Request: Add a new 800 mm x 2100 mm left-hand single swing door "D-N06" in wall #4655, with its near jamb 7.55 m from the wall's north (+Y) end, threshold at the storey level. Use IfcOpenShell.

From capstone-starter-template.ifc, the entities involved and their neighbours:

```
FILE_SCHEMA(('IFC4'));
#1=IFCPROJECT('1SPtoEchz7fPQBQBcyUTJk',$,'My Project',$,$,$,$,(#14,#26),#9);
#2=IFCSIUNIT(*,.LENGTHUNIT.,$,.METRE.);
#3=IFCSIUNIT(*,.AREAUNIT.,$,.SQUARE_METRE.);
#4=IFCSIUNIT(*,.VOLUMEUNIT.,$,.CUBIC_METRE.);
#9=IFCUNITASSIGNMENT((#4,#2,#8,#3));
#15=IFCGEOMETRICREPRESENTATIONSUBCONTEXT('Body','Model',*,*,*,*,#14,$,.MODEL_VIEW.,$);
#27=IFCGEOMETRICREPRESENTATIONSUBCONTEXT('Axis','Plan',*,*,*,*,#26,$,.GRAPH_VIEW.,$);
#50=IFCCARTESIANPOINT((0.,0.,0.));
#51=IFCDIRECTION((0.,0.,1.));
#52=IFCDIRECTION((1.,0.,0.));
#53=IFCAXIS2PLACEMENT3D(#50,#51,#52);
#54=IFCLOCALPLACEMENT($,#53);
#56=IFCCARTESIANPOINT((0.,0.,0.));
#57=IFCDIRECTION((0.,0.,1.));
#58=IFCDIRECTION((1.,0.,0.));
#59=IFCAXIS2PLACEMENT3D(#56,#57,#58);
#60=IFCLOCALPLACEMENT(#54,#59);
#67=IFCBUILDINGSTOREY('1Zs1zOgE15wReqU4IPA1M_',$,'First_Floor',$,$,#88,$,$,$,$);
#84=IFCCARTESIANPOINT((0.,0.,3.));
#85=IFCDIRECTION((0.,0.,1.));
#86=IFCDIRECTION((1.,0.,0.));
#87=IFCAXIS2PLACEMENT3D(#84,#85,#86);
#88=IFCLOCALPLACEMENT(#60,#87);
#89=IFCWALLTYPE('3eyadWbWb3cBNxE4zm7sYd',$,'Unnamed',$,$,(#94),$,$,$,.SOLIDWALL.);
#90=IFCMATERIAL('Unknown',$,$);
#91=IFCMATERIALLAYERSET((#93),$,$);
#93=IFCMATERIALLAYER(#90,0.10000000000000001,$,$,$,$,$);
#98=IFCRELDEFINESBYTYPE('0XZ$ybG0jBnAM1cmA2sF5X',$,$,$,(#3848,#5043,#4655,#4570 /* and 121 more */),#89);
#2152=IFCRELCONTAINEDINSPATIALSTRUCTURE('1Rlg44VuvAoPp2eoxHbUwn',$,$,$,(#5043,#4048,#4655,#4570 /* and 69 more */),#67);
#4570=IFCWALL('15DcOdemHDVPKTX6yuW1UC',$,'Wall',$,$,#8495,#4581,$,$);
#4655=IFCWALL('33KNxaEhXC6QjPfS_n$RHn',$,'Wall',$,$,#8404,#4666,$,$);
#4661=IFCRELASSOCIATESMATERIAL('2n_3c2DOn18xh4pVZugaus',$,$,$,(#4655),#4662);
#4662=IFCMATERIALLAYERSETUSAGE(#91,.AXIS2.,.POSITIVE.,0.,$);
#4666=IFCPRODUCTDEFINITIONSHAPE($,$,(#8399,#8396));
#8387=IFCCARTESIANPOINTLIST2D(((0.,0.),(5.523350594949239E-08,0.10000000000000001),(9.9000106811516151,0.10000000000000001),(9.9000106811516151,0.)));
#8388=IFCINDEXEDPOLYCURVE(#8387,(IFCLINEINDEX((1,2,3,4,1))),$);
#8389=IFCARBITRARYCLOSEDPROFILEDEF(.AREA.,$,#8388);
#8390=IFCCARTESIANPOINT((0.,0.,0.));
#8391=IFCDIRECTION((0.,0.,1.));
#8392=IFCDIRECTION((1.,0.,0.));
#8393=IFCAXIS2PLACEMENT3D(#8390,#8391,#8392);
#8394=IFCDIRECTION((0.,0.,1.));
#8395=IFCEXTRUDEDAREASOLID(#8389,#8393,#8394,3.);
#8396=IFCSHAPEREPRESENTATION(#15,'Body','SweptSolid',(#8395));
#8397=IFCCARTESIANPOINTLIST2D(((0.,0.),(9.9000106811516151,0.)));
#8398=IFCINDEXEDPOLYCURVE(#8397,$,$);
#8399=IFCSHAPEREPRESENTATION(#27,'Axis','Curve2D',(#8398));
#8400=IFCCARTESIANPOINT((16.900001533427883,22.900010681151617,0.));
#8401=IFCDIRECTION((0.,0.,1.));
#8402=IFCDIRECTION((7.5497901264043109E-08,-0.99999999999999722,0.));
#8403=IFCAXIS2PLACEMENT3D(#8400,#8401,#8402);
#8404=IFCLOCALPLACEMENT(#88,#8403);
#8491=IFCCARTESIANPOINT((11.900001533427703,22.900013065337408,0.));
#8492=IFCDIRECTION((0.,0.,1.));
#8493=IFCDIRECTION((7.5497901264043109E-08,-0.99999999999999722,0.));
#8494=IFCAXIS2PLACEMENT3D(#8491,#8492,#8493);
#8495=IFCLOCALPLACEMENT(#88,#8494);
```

```python
import numpy as np
import ifcopenshell
import ifcopenshell.api.feature
import ifcopenshell.api.geometry
import ifcopenshell.api.root
import ifcopenshell.api.spatial
import ifcopenshell.geom
import ifcopenshell.util.element
import ifcopenshell.util.placement
import ifcopenshell.util.representation
import ifcopenshell.util.shape
import ifcopenshell.util.unit

model = ifcopenshell.open("capstone-starter-template.ifc")
unit_scale = ifcopenshell.util.unit.calculate_unit_scale(model)
settings = ifcopenshell.geom.settings()


def volume(element):
    """Net volume in cubic metres, openings subtracted."""
    shape = ifcopenshell.geom.create_shape(settings, element)
    return ifcopenshell.util.shape.get_volume(shape.geometry)


wall = model.by_guid("33KNxaEhXC6QjPfS_n$RHn")
storey = ifcopenshell.util.element.get_container(wall, ifc_class="IfcBuildingStorey")
context = ifcopenshell.util.representation.get_context(model, "Model", "Body", "MODEL_VIEW")
before = volume(wall)

width, height, from_end, sill = 0.8, 2.1, 7.55, 0.0  # metres

# The wall runs along its own X axis, and the end named is its -X end.
wall_shape = ifcopenshell.geom.create_shape(settings, wall)
x, y, z = ifcopenshell.util.shape.get_vertices(wall_shape.geometry).T
start = x.min() + from_end
face, thickness = float(y.min()), float(y.max() - y.min())
wall_matrix = ifcopenshell.util.placement.get_local_placement(wall.ObjectPlacement)
level = ifcopenshell.util.placement.get_local_placement(storey.ObjectPlacement)[2, 3]


def in_wall(x, y):
    """Placement at x, y metres in the wall's axes, at sill height."""
    matrix = wall_matrix.copy()
    matrix[:, 3] = wall_matrix @ np.array([x / unit_scale, y / unit_scale, 0.0, 1.0])
    matrix[2, 3] = level + sill / unit_scale
    return matrix


# Opening: a box that overshoots both wall faces by 50 mm.
opening = ifcopenshell.api.root.create_entity(model, ifc_class="IfcOpeningElement", predefined_type="OPENING")
box = ifcopenshell.api.geometry.add_wall_representation(
    model, context=context, length=width, height=height, thickness=thickness + 0.1
)
ifcopenshell.api.geometry.assign_representation(model, product=opening, representation=box)
ifcopenshell.api.geometry.edit_object_placement(model, product=opening, matrix=in_wall(start, face - 0.05), is_si=False)
ifcopenshell.api.feature.add_feature(model, feature=opening, element=wall)

door = ifcopenshell.api.root.create_entity(model, ifc_class="IfcDoor", name="D-N06", predefined_type="DOOR")
door.OverallWidth, door.OverallHeight = width / unit_scale, height / unit_scale
door.OperationType = "SINGLE_SWING_LEFT"
body = ifcopenshell.api.geometry.add_door_representation(
    model,
    context=context,
    overall_width=door.OverallWidth,
    overall_height=door.OverallHeight,
    operation_type="SINGLE_SWING_LEFT",
    lining_properties={"LiningDepth": thickness / unit_scale, "ThresholdDepth": thickness / unit_scale},
)
ifcopenshell.api.geometry.assign_representation(model, product=door, representation=body)
ifcopenshell.api.spatial.assign_container(model, products=[door], relating_structure=storey)
ifcopenshell.api.feature.add_filling(model, opening=opening, element=door)

# The lining spans the wall, so the door starts at the wall face.
ifcopenshell.api.geometry.edit_object_placement(model, product=door, matrix=in_wall(start, face), is_si=False)

after = volume(wall)

print(f"wall volume {before:.3f} -> {after:.3f} m3")

model.write("capstone-starter-template_v2.ifc")
```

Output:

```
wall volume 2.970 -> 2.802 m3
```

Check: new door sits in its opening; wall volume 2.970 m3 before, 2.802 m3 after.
